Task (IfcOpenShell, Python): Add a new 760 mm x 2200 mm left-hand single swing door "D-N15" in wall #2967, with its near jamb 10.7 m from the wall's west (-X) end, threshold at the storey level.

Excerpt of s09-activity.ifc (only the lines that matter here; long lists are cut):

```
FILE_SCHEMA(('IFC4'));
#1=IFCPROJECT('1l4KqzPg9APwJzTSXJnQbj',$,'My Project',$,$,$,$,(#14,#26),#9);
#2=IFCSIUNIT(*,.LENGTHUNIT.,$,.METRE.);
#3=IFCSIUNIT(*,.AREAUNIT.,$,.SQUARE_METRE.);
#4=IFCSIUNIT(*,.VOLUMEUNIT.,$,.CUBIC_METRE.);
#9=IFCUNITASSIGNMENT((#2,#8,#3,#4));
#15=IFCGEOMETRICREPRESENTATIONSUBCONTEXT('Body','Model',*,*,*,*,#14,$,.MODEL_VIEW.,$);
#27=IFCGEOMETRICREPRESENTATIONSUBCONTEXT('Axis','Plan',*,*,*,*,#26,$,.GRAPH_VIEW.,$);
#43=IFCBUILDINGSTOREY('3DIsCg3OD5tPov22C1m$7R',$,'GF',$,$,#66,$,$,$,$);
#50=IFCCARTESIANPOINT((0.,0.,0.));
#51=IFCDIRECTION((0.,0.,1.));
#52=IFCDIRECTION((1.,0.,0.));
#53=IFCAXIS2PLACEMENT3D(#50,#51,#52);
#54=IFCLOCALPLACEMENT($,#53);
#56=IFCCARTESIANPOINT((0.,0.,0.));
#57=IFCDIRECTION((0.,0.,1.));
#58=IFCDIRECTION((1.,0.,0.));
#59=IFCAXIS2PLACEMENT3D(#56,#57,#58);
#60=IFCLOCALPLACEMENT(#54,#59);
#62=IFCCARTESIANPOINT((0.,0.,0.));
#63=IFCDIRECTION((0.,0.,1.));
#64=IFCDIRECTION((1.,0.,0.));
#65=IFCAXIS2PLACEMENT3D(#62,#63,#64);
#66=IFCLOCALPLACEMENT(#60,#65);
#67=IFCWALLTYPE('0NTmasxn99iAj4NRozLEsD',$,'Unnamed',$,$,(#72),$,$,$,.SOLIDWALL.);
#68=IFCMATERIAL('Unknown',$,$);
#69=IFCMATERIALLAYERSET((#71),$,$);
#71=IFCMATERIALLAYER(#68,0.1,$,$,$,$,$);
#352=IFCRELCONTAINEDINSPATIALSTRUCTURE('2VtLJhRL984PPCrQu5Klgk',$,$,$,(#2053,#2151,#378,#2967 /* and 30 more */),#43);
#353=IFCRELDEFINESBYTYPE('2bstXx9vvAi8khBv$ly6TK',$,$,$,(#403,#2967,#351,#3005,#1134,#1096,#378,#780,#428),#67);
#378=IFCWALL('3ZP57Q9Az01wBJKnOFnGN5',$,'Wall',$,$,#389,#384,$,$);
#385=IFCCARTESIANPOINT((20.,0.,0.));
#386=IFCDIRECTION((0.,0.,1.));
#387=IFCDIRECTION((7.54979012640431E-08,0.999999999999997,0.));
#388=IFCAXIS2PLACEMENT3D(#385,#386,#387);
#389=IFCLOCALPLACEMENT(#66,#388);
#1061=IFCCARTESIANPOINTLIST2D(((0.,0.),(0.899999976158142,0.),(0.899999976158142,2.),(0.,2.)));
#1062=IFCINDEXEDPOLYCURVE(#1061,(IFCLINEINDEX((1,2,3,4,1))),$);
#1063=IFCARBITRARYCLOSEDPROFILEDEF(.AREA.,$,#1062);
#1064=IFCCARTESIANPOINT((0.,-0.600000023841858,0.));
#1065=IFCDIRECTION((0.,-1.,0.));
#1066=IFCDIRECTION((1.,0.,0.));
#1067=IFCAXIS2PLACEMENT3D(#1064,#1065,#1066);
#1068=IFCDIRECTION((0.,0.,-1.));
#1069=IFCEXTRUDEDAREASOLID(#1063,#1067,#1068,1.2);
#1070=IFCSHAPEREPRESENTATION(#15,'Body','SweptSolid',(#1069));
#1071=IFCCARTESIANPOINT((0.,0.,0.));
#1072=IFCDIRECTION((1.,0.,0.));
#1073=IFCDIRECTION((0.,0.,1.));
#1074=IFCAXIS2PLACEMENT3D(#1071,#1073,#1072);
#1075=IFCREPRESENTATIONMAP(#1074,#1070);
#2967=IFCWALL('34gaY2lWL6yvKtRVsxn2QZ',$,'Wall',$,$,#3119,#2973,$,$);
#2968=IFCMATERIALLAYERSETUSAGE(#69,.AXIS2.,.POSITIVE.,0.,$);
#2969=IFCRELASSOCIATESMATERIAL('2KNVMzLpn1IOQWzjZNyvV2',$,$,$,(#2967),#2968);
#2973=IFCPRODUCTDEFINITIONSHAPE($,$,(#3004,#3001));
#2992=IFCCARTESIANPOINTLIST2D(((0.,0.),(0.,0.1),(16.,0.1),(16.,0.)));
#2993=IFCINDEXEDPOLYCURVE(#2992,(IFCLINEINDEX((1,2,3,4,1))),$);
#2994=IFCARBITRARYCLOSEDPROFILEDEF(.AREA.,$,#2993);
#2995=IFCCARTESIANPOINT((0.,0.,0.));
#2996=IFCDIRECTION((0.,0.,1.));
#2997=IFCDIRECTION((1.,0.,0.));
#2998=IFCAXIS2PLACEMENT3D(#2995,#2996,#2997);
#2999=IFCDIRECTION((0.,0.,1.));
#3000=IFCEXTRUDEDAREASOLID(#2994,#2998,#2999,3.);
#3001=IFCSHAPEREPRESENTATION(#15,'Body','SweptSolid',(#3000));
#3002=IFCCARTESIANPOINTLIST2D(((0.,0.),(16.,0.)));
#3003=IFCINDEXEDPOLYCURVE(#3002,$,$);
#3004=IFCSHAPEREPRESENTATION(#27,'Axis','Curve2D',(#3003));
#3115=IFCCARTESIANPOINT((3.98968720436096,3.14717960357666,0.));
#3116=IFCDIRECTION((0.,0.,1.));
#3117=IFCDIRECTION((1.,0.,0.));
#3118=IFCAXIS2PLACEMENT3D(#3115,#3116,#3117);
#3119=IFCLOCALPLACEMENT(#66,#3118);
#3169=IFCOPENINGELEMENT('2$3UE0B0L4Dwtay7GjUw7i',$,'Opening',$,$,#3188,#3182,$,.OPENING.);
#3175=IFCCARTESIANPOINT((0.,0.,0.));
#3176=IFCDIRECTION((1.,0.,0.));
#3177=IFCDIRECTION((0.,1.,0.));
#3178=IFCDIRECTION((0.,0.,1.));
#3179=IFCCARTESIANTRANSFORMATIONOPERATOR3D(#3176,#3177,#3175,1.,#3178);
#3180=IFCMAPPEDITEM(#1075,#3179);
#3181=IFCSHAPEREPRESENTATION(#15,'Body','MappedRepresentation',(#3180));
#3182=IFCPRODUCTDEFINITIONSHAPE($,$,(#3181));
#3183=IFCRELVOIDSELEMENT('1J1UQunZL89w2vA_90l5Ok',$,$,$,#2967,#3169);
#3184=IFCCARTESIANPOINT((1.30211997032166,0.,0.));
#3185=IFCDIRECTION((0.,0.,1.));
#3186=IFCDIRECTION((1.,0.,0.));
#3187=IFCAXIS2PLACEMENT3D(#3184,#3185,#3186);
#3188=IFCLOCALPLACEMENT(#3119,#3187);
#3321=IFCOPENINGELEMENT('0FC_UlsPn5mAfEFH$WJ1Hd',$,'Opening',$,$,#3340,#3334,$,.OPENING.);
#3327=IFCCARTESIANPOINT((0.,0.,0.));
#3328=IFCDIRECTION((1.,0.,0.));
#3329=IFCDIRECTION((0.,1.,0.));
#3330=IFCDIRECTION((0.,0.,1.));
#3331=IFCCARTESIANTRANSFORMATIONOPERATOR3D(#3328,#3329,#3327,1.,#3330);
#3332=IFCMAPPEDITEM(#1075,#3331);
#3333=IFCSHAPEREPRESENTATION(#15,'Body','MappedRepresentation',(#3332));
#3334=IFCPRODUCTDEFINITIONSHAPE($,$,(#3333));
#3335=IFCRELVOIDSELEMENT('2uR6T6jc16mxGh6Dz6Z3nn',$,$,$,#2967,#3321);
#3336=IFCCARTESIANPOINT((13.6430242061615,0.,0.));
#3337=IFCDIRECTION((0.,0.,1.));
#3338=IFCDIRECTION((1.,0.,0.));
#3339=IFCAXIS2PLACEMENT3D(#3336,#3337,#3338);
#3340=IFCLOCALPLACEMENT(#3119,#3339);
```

```python
import numpy as np
import ifcopenshell
import ifcopenshell.api.feature
import ifcopenshell.api.geometry
import ifcopenshell.api.root
import ifcopenshell.api.spatial
import ifcopenshell.geom
import ifcopenshell.util.element
import ifcopenshell.util.placement
import ifcopenshell.util.representation
import ifcopenshell.util.shape
import ifcopenshell.util.unit

model = ifcopenshell.open("s09-activity.ifc")
unit_scale = ifcopenshell.util.unit.calculate_unit_scale(model)
settings = ifcopenshell.geom.settings()


def volume(element):
    """Net volume in cubic metres, openings subtracted."""
    shape = ifcopenshell.geom.create_shape(settings, element)
    return ifcopenshell.util.shape.get_volume(shape.geometry)


wall = model.by_guid("34gaY2lWL6yvKtRVsxn2QZ")
storey = ifcopenshell.util.element.get_container(wall, ifc_class="IfcBuildingStorey")
context = ifcopenshell.util.representation.get_context(model, "Model", "Body", "MODEL_VIEW")
before = volume(wall)

width, height, from_end, sill = 0.76, 2.2, 10.7, 0.0  # metres

# The wall runs along its own X axis, and the end named is its -X end.
wall_shape = ifcopenshell.geom.create_shape(settings, wall)
x, y, z = ifcopenshell.util.shape.get_vertices(wall_shape.geometry).T
start = x.min() + from_end
face, thickness = float(y.min()), float(y.max() - y.min())
wall_matrix = ifcopenshell.util.placement.get_local_placement(wall.ObjectPlacement)
level = ifcopenshell.util.placement.get_local_placement(storey.ObjectPlacement)[2, 3]


def in_wall(x, y):
    """Placement at x, y metres in the wall's axes, at sill height."""
    matrix = wall_matrix.copy()
    matrix[:, 3] = wall_matrix @ np.array([x / unit_scale, y / unit_scale, 0.0, 1.0])
    matrix[2, 3] = level + sill / unit_scale
    return matrix


# Opening: a box that overshoots both wall faces by 50 mm.
opening = ifcopenshell.api.root.create_entity(model, ifc_class="IfcOpeningElement", predefined_type="OPENING")
box = ifcopenshell.api.geometry.add_wall_representation(
    model, context=context, length=width, height=height, thickness=thickness + 0.1
)
ifcopenshell.api.geometry.assign_representation(model, product=opening, representation=box)
ifcopenshell.api.geometry.edit_object_placement(model, product=opening, matrix=in_wall(start, face - 0.05), is_si=False)
ifcopenshell.api.feature.add_feature(model, feature=opening, element=wall)

door = ifcopenshell.api.root.create_entity(model, ifc_class="IfcDoor", name="D-N15", predefined_type="DOOR")
door.OverallWidth, door.OverallHeight = width / unit_scale, height / unit_scale
door.OperationType = "SINGLE_SWING_LEFT"
body = ifcopenshell.api.geometry.add_door_representation(
    model,
    context=context,
    overall_width=door.OverallWidth,
    overall_height=door.OverallHeight,
    operation_type="SINGLE_SWING_LEFT",
    lining_properties={"LiningDepth": thickness / unit_scale, "ThresholdDepth": thickness / unit_scale},
)
ifcopenshell.api.geometry.assign_representation(model, product=door, representation=body)
ifcopenshell.api.spatial.assign_container(model, products=[door], relating_structure=storey)
ifcopenshell.api.feature.add_filling(model, opening=opening, element=door)

# The lining spans the wall, so the door starts at the wall face.
ifcopenshell.api.geometry.edit_object_placement(model, product=door, matrix=in_wall(start, face), is_si=False)

after = volume(wall)

print(f"wall volume {before:.3f} -> {after:.3f} m3")

model.write("s09-activity-out.ifc")
```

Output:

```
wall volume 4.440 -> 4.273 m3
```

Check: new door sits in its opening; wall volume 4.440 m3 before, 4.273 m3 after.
